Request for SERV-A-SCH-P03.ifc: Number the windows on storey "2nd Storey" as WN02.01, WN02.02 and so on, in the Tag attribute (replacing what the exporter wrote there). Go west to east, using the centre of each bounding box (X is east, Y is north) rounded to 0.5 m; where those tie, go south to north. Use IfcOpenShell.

First a look at what the model holds.

```python
import ifcopenshell
import ifcopenshell.util.element
import ifcopenshell.util.placement

model = ifcopenshell.open("SERV-A-SCH-P03.ifc")
print(model.schema)
storey = next(s for s in model.by_type("IfcBuildingStorey") if s.Name == "2nd Storey")
windows = [e for e in ifcopenshell.util.element.get_decomposition(storey) if e.is_a("IfcWindow")]
for e in sorted(windows, key=lambda e: e.id()):
    origin = ifcopenshell.util.placement.get_local_placement(e.ObjectPlacement)[:3, 3]
    print(e.id(), e.Tag, e.Name, origin.round(2) + 0.0, sep=" | ")
```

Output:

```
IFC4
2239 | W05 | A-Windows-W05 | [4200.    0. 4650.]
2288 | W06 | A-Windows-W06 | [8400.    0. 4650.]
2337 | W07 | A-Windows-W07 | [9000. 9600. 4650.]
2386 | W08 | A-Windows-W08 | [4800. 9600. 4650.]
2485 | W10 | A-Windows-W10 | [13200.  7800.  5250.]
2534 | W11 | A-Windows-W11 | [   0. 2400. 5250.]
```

```python
import ifcopenshell
import ifcopenshell.geom
import ifcopenshell.util.element
import ifcopenshell.util.shape

model = ifcopenshell.open("SERV-A-SCH-P03.ifc")
settings = ifcopenshell.geom.settings()
settings.set("use-world-coords", True)


def centre(element):
    shape = ifcopenshell.geom.create_shape(settings, element)
    return ifcopenshell.util.shape.get_bbox_centroid(shape.geometry)


storey = next(s for s in model.by_type("IfcBuildingStorey") if s.Name == "2nd Storey")
windows = [e for e in ifcopenshell.util.element.get_decomposition(storey) if e.is_a("IfcWindow")]

# Insertion points can sit at a corner or the storey origin, so sort by the geometry (in metres).
centres = {e: centre(e) for e in windows}
windows.sort(key=lambda e: (round(centres[e][0] / 0.5), centres[e][1]))

for i, e in enumerate(windows, start=1):
    number = f"WN02.{i:02d}"
    e.Tag = number
    print(e.id(), number)

model.write("SERV-A-SCH-P03_edited.ifc")
```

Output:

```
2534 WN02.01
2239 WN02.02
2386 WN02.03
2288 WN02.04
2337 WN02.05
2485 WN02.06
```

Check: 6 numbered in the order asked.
